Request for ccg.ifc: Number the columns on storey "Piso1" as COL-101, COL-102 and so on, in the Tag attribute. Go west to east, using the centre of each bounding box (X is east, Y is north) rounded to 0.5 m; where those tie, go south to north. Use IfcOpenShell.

First a look at what the model holds.

```python
import ifcopenshell
import ifcopenshell.util.element
import ifcopenshell.util.placement

model = ifcopenshell.open("ccg.ifc")
print(model.schema)
storey = next(s for s in model.by_type("IfcBuildingStorey") if s.Name == "Piso1")
columns = [e for e in ifcopenshell.util.element.get_decomposition(storey) if e.is_a("IfcColumn")]
for e in sorted(columns, key=lambda e: e.id()):
    origin = ifcopenshell.util.placement.get_local_placement(e.ObjectPlacement)[:3, 3]
    print(e.id(), e.Tag, e.Name, origin.round(2) + 0.0, sep=" | ")
```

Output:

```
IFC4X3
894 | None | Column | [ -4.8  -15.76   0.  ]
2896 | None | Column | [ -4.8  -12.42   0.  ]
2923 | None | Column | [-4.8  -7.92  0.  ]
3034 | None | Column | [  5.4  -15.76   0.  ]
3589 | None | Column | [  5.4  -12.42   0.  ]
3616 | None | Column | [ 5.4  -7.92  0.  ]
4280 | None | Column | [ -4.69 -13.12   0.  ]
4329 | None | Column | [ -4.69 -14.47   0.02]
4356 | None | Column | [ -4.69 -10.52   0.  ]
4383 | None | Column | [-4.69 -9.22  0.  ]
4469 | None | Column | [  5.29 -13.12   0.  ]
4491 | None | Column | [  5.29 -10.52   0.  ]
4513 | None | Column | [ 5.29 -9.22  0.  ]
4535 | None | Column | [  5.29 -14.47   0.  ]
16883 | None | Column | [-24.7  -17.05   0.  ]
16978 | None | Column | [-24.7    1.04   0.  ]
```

```python
import ifcopenshell
import ifcopenshell.geom
import ifcopenshell.util.element
import ifcopenshell.util.shape

model = ifcopenshell.open("ccg.ifc")
settings = ifcopenshell.geom.settings()
settings.set("use-world-coords", True)


def centre(element):
    shape = ifcopenshell.geom.create_shape(settings, element)
    return ifcopenshell.util.shape.get_bbox_centroid(shape.geometry)


storey = next(s for s in model.by_type("IfcBuildingStorey") if s.Name == "Piso1")
columns = [e for e in ifcopenshell.util.element.get_decomposition(storey) if e.is_a("IfcColumn")]

# Insertion points can sit at a corner or the storey origin, so sort by the geometry (in metres).
centres = {e: centre(e) for e in columns}
columns.sort(key=lambda e: (round(centres[e][0] / 0.5), centres[e][1]))

for i, e in enumerate(columns, start=1):
    number = f"COL-1{i:02d}"
    e.Tag = number
    print(e.id(), number)

model.write("ccg_rev.ifc")
```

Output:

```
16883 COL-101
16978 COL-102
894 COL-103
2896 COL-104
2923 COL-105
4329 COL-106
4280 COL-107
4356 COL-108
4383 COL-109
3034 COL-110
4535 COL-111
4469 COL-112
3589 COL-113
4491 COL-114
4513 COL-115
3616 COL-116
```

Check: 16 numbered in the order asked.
